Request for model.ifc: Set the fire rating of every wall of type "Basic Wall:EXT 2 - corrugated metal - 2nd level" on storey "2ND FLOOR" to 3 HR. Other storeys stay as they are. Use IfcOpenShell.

First a look at what the model holds.

```python
import ifcopenshell
import ifcopenshell.util.element

model = ifcopenshell.open("model.ifc")
print(model.schema)
storey = next(s for s in model.by_type("IfcBuildingStorey") if s.Name == "2ND FLOOR")
walls = [e for e in ifcopenshell.util.element.get_decomposition(storey) if e.is_a("IfcWall")]
seen = {}
for e in walls:
    element_type = ifcopenshell.util.element.get_type(e)
    key = (element_type.Name if element_type != e and element_type else None, ifcopenshell.util.element.get_pset(e, "Pset_WallCommon", "FireRating"))
    seen[key] = seen.get(key, 0) + 1
for (name, value), count in sorted(seen.items(), key=str):
    print(count, "x", name, "|", value)
```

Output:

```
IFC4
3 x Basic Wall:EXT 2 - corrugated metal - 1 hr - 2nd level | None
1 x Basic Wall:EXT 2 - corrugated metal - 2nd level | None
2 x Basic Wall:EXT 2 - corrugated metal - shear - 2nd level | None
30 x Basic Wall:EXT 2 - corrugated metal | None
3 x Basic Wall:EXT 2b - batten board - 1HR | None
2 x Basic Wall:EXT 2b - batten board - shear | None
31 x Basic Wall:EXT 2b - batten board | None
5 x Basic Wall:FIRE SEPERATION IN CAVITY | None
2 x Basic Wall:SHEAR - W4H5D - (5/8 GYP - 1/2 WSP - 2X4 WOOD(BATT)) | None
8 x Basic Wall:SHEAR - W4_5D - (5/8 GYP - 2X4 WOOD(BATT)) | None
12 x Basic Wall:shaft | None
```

```python
import ifcopenshell
import ifcopenshell.api.pset
import ifcopenshell.util.element

model = ifcopenshell.open("model.ifc")

storey = next(s for s in model.by_type("IfcBuildingStorey") if s.Name == "2ND FLOOR")
walls = [e for e in ifcopenshell.util.element.get_decomposition(storey) if e.is_a("IfcWall")]

count = 0
for e in walls:
    element_type = ifcopenshell.util.element.get_type(e)
    if element_type in (None, e) or element_type.Name != "Basic Wall:EXT 2 - corrugated metal - 2nd level":
        continue
    # add_pset returns the element's existing set when there is one.
    pset = ifcopenshell.api.pset.add_pset(model, product=e, name="Pset_WallCommon")
    ifcopenshell.api.pset.edit_pset(model, pset=pset, properties={"FireRating": "3 HR"})
    count += 1

print(count, "walls updated")

model.write("model_v2.ifc")
```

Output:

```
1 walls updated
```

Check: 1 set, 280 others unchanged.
